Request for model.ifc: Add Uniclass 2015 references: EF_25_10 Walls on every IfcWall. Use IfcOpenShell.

First a look at what the model holds.

```python
import ifcopenshell

model = ifcopenshell.open("model.ifc")
print(model.schema)
print("classifications:", [c.Name for c in model.by_type("IfcClassification")])
for ifc_class in ("IfcDoor", "IfcRoof", "IfcStair", "IfcWall", "IfcWindow"):
    print(ifc_class, len(model.by_type(ifc_class)))
```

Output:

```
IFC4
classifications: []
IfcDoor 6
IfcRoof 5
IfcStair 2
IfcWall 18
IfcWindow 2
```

```python
import ifcopenshell
import ifcopenshell.api.classification

model = ifcopenshell.open("model.ifc")

system = ifcopenshell.api.classification.add_classification(model, classification="Uniclass 2015")

codes = {
    "IfcWall": ("EF_25_10", "Walls"),
}
for ifc_class, (code, name) in codes.items():
    products = model.by_type(ifc_class)
    ifcopenshell.api.classification.add_reference(
        model, products=products, classification=system, identification=code, name=name
    )
    print(code, len(products))

model.write("model-out.ifc")
```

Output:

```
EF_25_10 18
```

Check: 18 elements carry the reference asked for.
